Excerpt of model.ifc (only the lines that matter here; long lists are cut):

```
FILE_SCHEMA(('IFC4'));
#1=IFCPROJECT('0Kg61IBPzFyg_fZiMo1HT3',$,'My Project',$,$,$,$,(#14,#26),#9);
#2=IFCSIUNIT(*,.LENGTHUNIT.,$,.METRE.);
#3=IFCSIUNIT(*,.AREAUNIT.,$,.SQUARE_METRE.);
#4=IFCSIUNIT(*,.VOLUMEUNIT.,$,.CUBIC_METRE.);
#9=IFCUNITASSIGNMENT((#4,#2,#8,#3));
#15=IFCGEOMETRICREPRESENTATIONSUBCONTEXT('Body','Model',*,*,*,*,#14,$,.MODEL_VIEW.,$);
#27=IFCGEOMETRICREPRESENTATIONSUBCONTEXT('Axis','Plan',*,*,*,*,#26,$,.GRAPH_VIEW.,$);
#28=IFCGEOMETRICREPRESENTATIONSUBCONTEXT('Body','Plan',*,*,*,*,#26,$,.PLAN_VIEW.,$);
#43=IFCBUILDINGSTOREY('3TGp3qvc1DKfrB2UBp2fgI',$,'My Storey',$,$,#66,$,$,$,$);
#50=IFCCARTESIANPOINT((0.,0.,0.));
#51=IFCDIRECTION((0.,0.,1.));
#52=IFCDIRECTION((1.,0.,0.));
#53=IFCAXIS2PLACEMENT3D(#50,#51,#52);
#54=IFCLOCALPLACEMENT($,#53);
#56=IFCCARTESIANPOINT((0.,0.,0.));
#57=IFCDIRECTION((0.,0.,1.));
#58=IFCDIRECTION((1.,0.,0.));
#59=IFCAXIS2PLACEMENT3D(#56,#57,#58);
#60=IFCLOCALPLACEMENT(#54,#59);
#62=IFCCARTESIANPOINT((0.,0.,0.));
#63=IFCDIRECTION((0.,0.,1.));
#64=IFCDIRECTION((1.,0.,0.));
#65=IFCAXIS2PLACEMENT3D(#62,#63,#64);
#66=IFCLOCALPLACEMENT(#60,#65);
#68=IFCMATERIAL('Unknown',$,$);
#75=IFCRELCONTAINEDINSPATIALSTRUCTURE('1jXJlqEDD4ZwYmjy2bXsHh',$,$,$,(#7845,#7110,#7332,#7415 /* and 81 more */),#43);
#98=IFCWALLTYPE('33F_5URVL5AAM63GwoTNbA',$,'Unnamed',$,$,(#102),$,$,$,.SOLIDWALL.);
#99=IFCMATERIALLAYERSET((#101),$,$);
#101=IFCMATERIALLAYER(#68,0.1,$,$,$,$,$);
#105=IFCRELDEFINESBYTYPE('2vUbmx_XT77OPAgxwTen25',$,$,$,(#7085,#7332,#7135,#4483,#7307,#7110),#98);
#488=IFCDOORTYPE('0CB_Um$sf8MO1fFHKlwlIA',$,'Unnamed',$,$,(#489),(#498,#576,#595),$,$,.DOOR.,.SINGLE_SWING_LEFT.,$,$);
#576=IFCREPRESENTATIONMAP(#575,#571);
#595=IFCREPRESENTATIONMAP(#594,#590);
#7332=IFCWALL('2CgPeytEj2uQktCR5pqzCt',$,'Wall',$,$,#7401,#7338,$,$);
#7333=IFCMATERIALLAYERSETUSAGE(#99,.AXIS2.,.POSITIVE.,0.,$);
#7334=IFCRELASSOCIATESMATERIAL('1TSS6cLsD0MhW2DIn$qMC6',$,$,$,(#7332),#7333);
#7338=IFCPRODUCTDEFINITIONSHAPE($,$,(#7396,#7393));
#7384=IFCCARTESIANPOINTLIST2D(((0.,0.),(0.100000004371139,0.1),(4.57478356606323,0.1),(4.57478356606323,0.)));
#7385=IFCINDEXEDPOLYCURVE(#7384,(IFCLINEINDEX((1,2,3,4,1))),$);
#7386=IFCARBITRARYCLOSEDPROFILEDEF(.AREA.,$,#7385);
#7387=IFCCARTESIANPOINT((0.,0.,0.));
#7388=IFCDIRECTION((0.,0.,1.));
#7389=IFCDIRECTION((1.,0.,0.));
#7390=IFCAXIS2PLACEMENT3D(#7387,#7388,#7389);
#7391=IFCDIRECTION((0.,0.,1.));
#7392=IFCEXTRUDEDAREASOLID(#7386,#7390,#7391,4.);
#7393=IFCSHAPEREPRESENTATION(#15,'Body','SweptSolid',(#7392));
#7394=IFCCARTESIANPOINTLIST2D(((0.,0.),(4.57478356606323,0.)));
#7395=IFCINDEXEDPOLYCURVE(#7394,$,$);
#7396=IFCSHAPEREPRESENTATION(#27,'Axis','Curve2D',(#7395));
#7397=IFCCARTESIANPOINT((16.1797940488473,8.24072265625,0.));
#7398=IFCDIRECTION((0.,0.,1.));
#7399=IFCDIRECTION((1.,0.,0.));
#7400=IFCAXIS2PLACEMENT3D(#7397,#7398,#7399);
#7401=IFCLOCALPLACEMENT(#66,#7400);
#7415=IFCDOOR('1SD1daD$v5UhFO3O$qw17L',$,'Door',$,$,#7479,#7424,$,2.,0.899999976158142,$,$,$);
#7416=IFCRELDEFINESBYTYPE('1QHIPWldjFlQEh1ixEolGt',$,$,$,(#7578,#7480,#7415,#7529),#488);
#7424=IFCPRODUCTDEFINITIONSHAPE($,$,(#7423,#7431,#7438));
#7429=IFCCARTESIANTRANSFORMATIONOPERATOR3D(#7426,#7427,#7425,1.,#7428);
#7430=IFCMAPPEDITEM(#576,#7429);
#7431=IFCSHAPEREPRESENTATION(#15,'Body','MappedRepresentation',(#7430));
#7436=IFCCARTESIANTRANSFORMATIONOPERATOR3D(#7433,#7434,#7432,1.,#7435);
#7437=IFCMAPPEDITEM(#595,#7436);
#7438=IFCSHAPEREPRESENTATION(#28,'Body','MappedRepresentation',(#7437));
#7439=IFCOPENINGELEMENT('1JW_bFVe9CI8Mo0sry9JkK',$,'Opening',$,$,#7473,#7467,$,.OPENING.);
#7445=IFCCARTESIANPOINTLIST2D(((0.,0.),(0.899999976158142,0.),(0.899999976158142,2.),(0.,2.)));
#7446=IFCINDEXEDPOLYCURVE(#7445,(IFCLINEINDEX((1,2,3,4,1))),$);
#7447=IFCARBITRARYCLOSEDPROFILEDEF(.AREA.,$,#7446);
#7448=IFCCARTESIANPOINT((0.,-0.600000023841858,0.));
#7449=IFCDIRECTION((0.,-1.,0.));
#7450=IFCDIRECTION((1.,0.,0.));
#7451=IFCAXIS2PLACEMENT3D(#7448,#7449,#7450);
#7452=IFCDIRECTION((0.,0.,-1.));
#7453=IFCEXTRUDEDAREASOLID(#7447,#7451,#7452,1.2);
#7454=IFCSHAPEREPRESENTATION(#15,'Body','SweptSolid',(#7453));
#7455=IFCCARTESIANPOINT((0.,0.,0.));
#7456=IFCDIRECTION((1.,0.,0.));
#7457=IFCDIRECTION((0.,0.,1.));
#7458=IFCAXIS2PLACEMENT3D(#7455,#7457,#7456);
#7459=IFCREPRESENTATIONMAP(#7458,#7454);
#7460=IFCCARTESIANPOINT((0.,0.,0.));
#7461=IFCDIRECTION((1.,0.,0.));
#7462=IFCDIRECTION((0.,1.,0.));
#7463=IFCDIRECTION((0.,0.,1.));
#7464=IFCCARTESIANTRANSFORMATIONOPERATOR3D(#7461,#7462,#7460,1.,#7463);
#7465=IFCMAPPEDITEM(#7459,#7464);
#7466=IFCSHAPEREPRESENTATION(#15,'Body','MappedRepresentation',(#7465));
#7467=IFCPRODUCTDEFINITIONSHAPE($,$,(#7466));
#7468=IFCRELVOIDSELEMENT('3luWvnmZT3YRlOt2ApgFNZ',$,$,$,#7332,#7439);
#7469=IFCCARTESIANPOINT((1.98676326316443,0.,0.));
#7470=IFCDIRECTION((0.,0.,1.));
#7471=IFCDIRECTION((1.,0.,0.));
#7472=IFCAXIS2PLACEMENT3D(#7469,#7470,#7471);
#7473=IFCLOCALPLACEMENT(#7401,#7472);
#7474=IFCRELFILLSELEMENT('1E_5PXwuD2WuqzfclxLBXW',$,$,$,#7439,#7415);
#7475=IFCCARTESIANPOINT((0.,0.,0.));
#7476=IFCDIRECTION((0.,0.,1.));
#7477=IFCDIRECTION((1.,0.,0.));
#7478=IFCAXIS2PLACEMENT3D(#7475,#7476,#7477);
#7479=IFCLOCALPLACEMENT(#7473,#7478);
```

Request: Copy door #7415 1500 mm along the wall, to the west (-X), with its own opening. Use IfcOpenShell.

```python
import ifcopenshell
import ifcopenshell.api.feature
import ifcopenshell.api.geometry
import ifcopenshell.api.root
import ifcopenshell.geom
import ifcopenshell.util.element
import ifcopenshell.util.placement
import ifcopenshell.util.shape
import ifcopenshell.util.unit

model = ifcopenshell.open("model.ifc")
unit_scale = ifcopenshell.util.unit.calculate_unit_scale(model)
settings = ifcopenshell.geom.settings()


def volume(element):
    """Net volume in cubic metres, openings subtracted."""
    shape = ifcopenshell.geom.create_shape(settings, element)
    return ifcopenshell.util.shape.get_volume(shape.geometry)


door = model.by_id(7415)
opening = door.FillsVoids[0].RelatingOpeningElement
wall = opening.VoidsElements[0].RelatingBuildingElement
before = volume(wall)
shift = ifcopenshell.util.placement.get_local_placement(wall.ObjectPlacement)[:3, 0] * -1.5 / unit_scale

# copy_class copies the void relationship, type, container and properties, but no geometry.
new_opening = ifcopenshell.api.root.copy_class(model, product=opening)
new_opening.Representation = ifcopenshell.util.element.copy_deep(
    model, opening.Representation, exclude=["IfcGeometricRepresentationContext", "IfcRepresentationMap"]
)
new_door = ifcopenshell.api.root.copy_class(model, product=door)
new_door.Representation = ifcopenshell.util.element.copy_deep(
    model, door.Representation, exclude=["IfcGeometricRepresentationContext", "IfcRepresentationMap"]
)
ifcopenshell.api.feature.add_filling(model, opening=new_opening, element=new_door)

for old, new in ((opening, new_opening), (door, new_door)):
    matrix = ifcopenshell.util.placement.get_local_placement(old.ObjectPlacement)
    matrix[:3, 3] += shift
    ifcopenshell.api.geometry.edit_object_placement(model, product=new, matrix=matrix, is_si=False)

after = volume(wall)

print(f"wall volume {before:.3f} -> {after:.3f} m3")

model.write("model-out.ifc")
```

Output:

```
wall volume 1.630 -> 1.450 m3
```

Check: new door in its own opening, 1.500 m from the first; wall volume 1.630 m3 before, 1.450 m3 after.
